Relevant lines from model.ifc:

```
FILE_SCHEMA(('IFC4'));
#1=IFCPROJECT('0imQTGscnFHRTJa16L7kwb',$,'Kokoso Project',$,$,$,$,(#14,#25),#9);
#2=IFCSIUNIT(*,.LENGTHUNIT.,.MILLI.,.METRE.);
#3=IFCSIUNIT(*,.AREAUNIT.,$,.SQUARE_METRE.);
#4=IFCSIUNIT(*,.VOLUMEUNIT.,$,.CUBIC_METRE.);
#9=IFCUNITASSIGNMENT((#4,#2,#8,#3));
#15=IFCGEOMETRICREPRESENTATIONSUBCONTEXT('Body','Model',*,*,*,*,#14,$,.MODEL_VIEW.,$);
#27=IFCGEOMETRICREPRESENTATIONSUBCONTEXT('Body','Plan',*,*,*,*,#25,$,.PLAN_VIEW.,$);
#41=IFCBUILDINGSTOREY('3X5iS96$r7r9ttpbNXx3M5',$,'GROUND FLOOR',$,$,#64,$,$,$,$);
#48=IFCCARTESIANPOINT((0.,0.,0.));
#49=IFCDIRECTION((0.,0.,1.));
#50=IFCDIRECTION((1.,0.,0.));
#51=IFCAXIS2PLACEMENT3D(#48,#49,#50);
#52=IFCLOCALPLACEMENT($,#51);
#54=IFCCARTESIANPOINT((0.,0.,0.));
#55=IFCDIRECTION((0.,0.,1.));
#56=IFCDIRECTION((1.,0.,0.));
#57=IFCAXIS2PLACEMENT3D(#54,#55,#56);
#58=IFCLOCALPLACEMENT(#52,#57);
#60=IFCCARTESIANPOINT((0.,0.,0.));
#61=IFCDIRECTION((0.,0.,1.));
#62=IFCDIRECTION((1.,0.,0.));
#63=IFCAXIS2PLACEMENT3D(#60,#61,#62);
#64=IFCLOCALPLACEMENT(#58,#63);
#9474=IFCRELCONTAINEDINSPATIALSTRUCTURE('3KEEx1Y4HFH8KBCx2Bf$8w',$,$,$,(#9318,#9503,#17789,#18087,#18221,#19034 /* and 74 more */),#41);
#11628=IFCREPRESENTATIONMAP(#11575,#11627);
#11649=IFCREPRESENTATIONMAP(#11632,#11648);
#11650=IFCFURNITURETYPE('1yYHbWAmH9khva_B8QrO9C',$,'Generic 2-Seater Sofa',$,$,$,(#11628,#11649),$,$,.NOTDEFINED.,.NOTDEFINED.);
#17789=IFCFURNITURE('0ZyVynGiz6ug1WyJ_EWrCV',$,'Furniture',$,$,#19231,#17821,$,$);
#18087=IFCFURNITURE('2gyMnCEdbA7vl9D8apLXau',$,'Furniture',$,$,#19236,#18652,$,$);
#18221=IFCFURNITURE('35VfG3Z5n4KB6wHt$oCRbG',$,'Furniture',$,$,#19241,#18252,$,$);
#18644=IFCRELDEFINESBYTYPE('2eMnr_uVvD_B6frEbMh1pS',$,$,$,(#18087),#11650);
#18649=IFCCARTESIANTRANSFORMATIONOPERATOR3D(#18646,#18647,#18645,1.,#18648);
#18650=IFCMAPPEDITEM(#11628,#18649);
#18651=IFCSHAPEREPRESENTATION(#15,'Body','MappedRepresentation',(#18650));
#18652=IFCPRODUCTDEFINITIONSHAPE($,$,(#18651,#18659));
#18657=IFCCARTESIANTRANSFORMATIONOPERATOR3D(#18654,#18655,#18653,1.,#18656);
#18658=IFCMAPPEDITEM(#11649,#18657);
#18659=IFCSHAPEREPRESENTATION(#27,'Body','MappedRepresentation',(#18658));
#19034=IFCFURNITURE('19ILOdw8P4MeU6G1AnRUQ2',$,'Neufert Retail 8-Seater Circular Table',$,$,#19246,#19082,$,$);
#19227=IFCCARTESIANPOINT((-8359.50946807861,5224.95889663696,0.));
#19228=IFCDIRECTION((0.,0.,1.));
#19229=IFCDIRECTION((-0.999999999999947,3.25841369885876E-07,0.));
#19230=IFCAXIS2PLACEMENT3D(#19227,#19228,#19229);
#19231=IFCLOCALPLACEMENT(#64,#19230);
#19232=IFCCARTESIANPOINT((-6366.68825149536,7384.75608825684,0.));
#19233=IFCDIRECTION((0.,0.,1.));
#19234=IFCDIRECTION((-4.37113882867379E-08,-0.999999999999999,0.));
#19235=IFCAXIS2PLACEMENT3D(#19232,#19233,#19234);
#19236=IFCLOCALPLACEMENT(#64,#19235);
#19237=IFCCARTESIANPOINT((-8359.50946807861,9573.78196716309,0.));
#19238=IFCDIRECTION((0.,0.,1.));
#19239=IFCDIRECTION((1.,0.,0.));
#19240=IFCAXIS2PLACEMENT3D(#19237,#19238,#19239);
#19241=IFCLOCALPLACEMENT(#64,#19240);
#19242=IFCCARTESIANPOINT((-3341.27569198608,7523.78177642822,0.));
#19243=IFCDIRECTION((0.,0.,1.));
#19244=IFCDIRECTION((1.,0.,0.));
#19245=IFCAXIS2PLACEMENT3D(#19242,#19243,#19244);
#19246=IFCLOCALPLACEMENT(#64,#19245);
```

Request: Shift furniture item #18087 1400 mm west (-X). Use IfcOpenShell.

```python
import ifcopenshell
import ifcopenshell.api.geometry
import ifcopenshell.util.placement
import ifcopenshell.util.unit

model = ifcopenshell.open("model.ifc")
unit_scale = ifcopenshell.util.unit.calculate_unit_scale(model)

item = model.by_guid("2gyMnCEdbA7vl9D8apLXau")
matrix = ifcopenshell.util.placement.get_local_placement(item.ObjectPlacement)
matrix[0, 3] -= 1.4 / unit_scale
ifcopenshell.api.geometry.edit_object_placement(model, product=item, matrix=matrix, is_si=False)

print(ifcopenshell.util.placement.get_local_placement(item.ObjectPlacement).round(3) + 0.0)

model.write("model_edited.ifc")
```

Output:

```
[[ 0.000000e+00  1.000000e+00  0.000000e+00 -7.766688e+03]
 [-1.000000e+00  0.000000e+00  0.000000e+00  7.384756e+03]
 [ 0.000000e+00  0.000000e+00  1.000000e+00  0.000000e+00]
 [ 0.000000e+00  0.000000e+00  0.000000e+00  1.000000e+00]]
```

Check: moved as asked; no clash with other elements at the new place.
